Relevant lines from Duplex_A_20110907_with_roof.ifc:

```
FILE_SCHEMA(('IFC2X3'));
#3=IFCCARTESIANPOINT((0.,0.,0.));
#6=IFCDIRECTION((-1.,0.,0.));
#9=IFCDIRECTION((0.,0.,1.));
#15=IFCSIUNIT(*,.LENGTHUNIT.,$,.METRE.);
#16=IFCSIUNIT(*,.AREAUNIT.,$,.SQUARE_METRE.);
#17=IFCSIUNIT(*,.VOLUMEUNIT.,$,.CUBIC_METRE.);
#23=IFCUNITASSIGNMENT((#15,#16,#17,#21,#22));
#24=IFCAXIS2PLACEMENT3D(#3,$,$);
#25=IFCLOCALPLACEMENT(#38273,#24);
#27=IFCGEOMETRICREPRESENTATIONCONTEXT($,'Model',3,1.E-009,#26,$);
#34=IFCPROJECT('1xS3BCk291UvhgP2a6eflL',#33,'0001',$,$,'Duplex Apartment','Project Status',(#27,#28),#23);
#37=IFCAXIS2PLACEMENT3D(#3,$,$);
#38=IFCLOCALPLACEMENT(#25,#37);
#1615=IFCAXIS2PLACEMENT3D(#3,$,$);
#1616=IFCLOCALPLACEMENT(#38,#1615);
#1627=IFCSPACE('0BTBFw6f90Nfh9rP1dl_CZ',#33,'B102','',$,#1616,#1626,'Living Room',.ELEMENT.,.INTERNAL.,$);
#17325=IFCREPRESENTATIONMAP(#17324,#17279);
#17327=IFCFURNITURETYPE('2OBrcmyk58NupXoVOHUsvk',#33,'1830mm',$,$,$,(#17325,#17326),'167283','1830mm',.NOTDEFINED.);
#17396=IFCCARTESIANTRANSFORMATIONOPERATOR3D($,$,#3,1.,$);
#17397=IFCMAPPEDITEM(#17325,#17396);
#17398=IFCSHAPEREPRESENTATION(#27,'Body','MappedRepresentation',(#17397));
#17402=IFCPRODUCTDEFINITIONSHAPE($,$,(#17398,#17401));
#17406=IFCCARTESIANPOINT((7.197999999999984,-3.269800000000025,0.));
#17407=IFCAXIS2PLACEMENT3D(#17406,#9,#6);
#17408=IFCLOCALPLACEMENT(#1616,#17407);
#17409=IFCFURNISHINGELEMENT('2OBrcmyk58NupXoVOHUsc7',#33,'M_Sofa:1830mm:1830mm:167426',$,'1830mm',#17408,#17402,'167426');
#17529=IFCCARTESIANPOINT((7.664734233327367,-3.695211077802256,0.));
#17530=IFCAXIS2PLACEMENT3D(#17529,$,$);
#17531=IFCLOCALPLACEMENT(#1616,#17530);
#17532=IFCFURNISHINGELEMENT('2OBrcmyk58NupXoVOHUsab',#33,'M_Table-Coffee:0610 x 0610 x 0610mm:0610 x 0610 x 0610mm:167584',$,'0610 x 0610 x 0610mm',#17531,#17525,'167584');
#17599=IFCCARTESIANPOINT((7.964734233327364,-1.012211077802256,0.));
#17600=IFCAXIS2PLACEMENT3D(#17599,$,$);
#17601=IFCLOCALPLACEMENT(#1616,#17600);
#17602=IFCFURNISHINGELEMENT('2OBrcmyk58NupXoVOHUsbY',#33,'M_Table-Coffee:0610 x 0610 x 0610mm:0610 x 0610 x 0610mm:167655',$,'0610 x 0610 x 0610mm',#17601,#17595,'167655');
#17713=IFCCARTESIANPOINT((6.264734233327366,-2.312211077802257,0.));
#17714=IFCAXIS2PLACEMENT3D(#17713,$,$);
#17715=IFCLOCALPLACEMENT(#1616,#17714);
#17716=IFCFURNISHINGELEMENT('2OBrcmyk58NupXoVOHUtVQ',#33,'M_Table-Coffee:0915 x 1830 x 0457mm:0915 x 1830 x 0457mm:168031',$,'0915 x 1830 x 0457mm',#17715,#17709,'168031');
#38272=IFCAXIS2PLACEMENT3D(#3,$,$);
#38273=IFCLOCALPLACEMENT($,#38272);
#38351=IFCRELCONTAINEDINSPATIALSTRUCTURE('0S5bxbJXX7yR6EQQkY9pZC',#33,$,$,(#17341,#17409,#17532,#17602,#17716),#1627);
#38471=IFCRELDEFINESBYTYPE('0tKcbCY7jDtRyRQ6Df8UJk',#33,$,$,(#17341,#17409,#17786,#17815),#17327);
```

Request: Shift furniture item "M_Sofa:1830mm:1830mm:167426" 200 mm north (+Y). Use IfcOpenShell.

```python
import ifcopenshell
import ifcopenshell.api.geometry
import ifcopenshell.util.placement
import ifcopenshell.util.unit

model = ifcopenshell.open("Duplex_A_20110907_with_roof.ifc")
unit_scale = ifcopenshell.util.unit.calculate_unit_scale(model)

item = model.by_id(17409)
matrix = ifcopenshell.util.placement.get_local_placement(item.ObjectPlacement)
matrix[1, 3] += 0.2 / unit_scale
ifcopenshell.api.geometry.edit_object_placement(model, product=item, matrix=matrix, is_si=False)

print(ifcopenshell.util.placement.get_local_placement(item.ObjectPlacement).round(3) + 0.0)

model.write("Duplex_A_20110907_with_roof_rev.ifc")
```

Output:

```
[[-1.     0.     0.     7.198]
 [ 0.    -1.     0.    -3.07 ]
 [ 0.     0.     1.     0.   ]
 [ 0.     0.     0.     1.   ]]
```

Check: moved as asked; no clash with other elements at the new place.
